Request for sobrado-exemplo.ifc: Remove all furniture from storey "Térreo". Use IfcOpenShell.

First a look at what the model holds.

```python
import ifcopenshell
import ifcopenshell.util.element

model = ifcopenshell.open("sobrado-exemplo.ifc")
print(model.schema)
storey = next(s for s in model.by_type("IfcBuildingStorey") if s.Name == "Térreo")
furniture = [e for e in ifcopenshell.util.element.get_decomposition(storey) if e.is_a("IfcFurnishingElement")]
seen = {}
for e in furniture:
    element_type = ifcopenshell.util.element.get_type(e)
    name = element_type.Name if element_type not in (None, e) else None
    seen[name] = seen.get(name, 0) + 1
for name, count in sorted(seen.items(), key=str):
    print(count, "x", name)
```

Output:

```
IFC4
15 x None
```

```python
import ifcopenshell
import ifcopenshell.api.root
import ifcopenshell.util.element

model = ifcopenshell.open("sobrado-exemplo.ifc")

storey = next(s for s in model.by_type("IfcBuildingStorey") if s.Name == "Térreo")
furniture = [e for e in ifcopenshell.util.element.get_decomposition(storey) if e.is_a("IfcFurnishingElement")]

for e in furniture:
    ifcopenshell.api.root.remove_product(model, product=e)
print(len(furniture), "removed")

model.write("sobrado-exemplo_updated.ifc")
```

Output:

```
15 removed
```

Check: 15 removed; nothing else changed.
